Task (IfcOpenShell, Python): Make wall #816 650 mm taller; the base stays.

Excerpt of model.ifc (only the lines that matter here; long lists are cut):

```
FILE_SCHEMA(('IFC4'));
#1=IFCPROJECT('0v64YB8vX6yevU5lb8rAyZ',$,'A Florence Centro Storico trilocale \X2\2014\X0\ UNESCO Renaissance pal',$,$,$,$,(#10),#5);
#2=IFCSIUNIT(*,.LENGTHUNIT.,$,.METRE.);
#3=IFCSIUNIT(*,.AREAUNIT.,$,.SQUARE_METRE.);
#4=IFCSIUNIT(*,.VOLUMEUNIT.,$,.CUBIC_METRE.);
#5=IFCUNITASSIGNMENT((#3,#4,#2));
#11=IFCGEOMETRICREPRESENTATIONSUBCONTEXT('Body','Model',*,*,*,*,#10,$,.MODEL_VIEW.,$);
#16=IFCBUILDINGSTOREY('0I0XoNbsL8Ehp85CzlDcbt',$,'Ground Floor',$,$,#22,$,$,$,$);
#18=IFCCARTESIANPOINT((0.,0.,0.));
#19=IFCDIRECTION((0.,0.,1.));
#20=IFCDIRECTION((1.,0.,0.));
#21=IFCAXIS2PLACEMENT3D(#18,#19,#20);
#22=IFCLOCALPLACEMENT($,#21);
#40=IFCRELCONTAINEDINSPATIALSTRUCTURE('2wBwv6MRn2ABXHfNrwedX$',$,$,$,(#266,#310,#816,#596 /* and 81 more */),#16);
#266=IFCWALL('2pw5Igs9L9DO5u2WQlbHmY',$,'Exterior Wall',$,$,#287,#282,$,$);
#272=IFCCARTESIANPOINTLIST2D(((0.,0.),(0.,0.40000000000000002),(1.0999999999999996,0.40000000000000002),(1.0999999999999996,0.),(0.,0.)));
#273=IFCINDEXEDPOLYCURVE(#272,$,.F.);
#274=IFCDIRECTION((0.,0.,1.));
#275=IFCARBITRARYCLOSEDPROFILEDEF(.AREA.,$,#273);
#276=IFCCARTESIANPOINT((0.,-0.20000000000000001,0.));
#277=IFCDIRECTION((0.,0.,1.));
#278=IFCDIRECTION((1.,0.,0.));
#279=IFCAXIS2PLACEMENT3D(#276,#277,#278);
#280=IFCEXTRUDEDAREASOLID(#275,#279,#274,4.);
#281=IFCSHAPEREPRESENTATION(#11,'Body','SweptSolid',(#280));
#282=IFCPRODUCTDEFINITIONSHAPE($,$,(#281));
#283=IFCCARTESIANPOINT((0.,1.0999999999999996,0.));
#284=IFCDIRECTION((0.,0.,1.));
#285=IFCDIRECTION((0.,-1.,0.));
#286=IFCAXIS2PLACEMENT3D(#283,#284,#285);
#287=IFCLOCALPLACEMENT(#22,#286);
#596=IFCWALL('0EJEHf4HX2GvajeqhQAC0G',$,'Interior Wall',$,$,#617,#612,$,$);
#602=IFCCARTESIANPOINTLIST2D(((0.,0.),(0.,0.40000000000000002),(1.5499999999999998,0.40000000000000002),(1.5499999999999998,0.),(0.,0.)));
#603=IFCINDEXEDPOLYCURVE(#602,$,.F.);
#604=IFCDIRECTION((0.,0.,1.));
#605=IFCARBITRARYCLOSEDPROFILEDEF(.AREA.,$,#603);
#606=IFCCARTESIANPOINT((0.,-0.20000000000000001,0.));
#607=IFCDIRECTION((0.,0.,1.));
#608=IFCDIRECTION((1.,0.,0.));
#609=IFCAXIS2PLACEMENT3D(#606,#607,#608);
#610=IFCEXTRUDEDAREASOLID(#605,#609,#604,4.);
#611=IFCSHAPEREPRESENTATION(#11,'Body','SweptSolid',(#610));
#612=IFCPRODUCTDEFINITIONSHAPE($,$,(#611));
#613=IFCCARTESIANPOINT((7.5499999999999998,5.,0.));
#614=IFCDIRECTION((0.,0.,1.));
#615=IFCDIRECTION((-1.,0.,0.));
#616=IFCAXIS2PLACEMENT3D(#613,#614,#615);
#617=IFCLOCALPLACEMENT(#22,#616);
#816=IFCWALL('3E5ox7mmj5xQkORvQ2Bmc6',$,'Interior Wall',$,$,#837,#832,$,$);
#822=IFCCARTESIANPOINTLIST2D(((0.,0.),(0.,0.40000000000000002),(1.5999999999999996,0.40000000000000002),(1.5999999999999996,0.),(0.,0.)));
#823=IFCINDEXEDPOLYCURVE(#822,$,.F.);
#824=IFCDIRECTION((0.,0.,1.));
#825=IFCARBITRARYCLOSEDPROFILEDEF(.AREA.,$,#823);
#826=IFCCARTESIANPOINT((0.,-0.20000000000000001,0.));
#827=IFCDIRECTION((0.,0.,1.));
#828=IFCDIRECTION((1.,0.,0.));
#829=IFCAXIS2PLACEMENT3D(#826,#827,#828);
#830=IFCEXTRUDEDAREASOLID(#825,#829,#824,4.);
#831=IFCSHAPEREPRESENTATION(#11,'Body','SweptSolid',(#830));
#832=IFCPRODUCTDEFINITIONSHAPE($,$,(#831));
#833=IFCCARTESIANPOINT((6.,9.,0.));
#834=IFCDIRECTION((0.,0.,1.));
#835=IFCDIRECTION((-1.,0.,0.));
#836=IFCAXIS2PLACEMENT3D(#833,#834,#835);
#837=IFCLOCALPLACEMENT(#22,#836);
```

```python
import ifcopenshell
import ifcopenshell.geom
import ifcopenshell.util.representation
import ifcopenshell.util.shape

model = ifcopenshell.open("model.ifc")
settings = ifcopenshell.geom.settings()


def volume(element):
    """Net volume in cubic metres, openings subtracted."""
    shape = ifcopenshell.geom.create_shape(settings, element)
    return ifcopenshell.util.shape.get_volume(shape.geometry)


wall = model.by_guid("3E5ox7mmj5xQkORvQ2Bmc6")
before = volume(wall)

body = ifcopenshell.util.representation.get_representation(wall, "Model", "Body")
solid = body.Items[0]
old_height = solid.Depth
solid.Depth += 0.65
after = volume(wall)

print(f"height {old_height:g} -> {solid.Depth:g}, volume {before:.3f} -> {after:.3f} m3")

model.write("model_updated.ifc")
```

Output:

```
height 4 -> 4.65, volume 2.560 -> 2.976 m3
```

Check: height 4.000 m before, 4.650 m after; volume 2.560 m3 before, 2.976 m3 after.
